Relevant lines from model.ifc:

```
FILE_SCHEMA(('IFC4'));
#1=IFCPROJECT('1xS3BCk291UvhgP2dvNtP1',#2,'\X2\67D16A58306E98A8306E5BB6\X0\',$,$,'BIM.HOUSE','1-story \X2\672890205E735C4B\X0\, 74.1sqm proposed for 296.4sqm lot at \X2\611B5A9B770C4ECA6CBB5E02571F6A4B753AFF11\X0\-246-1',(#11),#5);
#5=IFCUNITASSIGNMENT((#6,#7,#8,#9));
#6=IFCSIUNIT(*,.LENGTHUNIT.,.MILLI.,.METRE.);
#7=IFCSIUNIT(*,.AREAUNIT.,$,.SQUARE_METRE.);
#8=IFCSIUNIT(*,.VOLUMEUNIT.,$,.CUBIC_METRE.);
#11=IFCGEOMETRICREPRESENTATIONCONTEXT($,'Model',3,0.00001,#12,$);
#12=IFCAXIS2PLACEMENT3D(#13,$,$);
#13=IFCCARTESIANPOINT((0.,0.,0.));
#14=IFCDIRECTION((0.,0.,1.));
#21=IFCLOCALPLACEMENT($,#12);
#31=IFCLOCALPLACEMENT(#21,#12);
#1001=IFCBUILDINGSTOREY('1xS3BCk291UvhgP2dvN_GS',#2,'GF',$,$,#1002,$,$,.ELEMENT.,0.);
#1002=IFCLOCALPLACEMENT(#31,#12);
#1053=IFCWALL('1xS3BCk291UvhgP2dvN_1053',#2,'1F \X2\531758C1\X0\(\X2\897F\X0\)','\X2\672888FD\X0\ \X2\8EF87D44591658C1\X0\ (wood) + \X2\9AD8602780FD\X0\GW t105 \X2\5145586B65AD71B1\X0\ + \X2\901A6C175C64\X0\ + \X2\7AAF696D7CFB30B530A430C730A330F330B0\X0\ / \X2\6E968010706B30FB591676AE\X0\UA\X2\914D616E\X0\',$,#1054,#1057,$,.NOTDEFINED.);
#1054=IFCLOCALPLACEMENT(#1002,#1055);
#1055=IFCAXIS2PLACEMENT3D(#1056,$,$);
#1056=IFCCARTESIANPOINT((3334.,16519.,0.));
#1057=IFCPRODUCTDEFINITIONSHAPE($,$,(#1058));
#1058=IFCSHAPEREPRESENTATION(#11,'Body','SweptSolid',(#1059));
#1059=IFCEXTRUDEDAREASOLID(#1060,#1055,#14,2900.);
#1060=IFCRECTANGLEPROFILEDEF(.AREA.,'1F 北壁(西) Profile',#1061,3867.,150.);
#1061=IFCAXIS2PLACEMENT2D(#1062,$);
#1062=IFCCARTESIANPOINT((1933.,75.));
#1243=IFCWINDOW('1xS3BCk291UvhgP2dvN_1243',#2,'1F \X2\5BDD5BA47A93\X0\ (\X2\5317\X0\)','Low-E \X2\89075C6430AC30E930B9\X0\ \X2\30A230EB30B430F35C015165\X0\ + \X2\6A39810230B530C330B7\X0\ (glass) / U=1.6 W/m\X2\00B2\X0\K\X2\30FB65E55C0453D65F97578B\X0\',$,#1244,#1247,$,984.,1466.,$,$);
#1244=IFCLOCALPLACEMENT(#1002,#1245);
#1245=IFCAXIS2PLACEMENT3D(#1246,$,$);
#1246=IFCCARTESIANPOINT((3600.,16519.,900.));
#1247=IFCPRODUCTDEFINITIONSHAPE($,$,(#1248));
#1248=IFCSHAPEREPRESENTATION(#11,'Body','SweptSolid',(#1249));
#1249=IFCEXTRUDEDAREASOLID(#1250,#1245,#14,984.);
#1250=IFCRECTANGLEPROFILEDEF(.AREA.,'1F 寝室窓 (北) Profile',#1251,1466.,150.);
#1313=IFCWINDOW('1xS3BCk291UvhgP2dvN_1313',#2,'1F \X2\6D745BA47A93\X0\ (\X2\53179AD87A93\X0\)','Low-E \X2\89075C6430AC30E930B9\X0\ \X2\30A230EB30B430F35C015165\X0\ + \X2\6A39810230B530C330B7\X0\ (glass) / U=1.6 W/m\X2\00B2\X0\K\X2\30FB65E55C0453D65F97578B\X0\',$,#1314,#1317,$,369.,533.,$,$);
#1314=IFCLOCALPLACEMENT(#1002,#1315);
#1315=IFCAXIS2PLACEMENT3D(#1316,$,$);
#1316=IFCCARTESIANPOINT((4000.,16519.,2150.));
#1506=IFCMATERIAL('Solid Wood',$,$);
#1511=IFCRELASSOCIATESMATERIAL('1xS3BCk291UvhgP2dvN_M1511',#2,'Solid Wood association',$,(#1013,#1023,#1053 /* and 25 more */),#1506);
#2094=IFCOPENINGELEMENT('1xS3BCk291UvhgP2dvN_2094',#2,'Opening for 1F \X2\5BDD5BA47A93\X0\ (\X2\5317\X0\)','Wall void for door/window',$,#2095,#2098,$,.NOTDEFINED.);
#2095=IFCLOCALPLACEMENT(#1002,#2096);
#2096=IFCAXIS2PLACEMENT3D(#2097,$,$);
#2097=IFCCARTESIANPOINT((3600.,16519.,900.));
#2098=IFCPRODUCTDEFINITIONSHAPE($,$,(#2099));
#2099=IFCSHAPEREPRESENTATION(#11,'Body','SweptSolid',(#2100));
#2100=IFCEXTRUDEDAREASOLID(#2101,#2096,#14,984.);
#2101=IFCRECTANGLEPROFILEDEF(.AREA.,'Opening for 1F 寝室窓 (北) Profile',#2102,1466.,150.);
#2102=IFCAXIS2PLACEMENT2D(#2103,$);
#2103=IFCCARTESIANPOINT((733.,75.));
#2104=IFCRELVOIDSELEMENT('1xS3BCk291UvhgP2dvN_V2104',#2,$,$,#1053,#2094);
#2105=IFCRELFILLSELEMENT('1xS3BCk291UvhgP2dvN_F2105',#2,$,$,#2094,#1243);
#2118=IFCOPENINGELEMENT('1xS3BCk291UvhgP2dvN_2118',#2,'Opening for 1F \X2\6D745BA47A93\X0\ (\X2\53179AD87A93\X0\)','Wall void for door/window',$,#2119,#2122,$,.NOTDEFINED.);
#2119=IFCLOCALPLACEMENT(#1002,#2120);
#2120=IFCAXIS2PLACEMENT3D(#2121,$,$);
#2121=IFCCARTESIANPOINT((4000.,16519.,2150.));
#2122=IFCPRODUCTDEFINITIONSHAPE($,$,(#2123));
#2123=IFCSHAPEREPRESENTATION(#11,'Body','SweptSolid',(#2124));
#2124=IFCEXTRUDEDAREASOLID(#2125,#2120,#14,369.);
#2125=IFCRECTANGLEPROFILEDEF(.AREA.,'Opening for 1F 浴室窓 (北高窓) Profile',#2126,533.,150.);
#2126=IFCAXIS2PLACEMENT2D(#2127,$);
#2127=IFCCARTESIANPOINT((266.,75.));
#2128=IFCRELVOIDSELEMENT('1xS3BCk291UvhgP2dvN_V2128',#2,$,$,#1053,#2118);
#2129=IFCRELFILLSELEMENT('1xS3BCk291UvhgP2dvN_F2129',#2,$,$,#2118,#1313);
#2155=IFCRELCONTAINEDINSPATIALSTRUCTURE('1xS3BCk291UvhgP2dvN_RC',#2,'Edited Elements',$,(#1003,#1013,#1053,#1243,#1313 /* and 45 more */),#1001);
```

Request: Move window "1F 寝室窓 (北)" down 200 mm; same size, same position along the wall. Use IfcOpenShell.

```python
import numpy as np
import ifcopenshell
import ifcopenshell.api.geometry
import ifcopenshell.util.placement
import ifcopenshell.util.unit

model = ifcopenshell.open("model.ifc")
unit_scale = ifcopenshell.util.unit.calculate_unit_scale(model)

window = model.by_guid("1xS3BCk291UvhgP2dvN_1243")
opening = window.FillsVoids[0].RelatingOpeningElement
dz = -0.2 / unit_scale

shift = np.array([0.0, 0.0, dz])
# The window is not placed relative to its opening, so move both.
for product in (opening, window):
    matrix = ifcopenshell.util.placement.get_local_placement(product.ObjectPlacement)
    matrix[:3, 3] += shift
    ifcopenshell.api.geometry.edit_object_placement(model, product=product, matrix=matrix, is_si=False)

print(f"moved by {dz * unit_scale:+.3f} m")

model.write("model-out.ifc")
```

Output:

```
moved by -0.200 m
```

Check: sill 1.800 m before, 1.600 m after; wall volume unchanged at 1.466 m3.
